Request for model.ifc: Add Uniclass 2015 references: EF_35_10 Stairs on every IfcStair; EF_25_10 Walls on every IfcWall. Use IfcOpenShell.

First a look at what the model holds.

```python
import ifcopenshell

model = ifcopenshell.open("model.ifc")
print(model.schema)
print("classifications:", [c.Name for c in model.by_type("IfcClassification")])
for ifc_class in ("IfcDoor", "IfcRoof", "IfcStair", "IfcWall", "IfcWindow"):
    print(ifc_class, len(model.by_type(ifc_class)))
```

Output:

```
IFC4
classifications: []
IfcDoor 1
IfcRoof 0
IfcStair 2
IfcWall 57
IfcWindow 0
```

```python
import ifcopenshell
import ifcopenshell.api.classification

model = ifcopenshell.open("model.ifc")

system = ifcopenshell.api.classification.add_classification(model, classification="Uniclass 2015")

codes = {
    "IfcStair": ("EF_35_10", "Stairs"),
    "IfcWall": ("EF_25_10", "Walls"),
}
for ifc_class, (code, name) in codes.items():
    products = model.by_type(ifc_class)
    ifcopenshell.api.classification.add_reference(
        model, products=products, classification=system, identification=code, name=name
    )
    print(code, len(products))

model.write("model-out.ifc")
```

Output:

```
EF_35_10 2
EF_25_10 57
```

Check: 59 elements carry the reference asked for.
